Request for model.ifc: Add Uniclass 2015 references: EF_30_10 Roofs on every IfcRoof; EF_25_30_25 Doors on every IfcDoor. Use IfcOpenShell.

First a look at what the model holds.

```python
import ifcopenshell

model = ifcopenshell.open("model.ifc")
print(model.schema)
print("classifications:", [c.Name for c in model.by_type("IfcClassification")])
for ifc_class in ("IfcDoor", "IfcRoof", "IfcStair", "IfcWall", "IfcWindow"):
    print(ifc_class, len(model.by_type(ifc_class)))
```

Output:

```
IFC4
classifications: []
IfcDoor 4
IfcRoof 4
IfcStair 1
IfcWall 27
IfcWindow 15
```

```python
import ifcopenshell
import ifcopenshell.api.classification

model = ifcopenshell.open("model.ifc")

system = ifcopenshell.api.classification.add_classification(model, classification="Uniclass 2015")

codes = {
    "IfcRoof": ("EF_30_10", "Roofs"),
    "IfcDoor": ("EF_25_30_25", "Doors"),
}
for ifc_class, (code, name) in codes.items():
    products = model.by_type(ifc_class)
    ifcopenshell.api.classification.add_reference(
        model, products=products, classification=system, identification=code, name=name
    )
    print(code, len(products))

model.write("model_updated.ifc")
```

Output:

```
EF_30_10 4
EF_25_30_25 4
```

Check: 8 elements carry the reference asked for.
